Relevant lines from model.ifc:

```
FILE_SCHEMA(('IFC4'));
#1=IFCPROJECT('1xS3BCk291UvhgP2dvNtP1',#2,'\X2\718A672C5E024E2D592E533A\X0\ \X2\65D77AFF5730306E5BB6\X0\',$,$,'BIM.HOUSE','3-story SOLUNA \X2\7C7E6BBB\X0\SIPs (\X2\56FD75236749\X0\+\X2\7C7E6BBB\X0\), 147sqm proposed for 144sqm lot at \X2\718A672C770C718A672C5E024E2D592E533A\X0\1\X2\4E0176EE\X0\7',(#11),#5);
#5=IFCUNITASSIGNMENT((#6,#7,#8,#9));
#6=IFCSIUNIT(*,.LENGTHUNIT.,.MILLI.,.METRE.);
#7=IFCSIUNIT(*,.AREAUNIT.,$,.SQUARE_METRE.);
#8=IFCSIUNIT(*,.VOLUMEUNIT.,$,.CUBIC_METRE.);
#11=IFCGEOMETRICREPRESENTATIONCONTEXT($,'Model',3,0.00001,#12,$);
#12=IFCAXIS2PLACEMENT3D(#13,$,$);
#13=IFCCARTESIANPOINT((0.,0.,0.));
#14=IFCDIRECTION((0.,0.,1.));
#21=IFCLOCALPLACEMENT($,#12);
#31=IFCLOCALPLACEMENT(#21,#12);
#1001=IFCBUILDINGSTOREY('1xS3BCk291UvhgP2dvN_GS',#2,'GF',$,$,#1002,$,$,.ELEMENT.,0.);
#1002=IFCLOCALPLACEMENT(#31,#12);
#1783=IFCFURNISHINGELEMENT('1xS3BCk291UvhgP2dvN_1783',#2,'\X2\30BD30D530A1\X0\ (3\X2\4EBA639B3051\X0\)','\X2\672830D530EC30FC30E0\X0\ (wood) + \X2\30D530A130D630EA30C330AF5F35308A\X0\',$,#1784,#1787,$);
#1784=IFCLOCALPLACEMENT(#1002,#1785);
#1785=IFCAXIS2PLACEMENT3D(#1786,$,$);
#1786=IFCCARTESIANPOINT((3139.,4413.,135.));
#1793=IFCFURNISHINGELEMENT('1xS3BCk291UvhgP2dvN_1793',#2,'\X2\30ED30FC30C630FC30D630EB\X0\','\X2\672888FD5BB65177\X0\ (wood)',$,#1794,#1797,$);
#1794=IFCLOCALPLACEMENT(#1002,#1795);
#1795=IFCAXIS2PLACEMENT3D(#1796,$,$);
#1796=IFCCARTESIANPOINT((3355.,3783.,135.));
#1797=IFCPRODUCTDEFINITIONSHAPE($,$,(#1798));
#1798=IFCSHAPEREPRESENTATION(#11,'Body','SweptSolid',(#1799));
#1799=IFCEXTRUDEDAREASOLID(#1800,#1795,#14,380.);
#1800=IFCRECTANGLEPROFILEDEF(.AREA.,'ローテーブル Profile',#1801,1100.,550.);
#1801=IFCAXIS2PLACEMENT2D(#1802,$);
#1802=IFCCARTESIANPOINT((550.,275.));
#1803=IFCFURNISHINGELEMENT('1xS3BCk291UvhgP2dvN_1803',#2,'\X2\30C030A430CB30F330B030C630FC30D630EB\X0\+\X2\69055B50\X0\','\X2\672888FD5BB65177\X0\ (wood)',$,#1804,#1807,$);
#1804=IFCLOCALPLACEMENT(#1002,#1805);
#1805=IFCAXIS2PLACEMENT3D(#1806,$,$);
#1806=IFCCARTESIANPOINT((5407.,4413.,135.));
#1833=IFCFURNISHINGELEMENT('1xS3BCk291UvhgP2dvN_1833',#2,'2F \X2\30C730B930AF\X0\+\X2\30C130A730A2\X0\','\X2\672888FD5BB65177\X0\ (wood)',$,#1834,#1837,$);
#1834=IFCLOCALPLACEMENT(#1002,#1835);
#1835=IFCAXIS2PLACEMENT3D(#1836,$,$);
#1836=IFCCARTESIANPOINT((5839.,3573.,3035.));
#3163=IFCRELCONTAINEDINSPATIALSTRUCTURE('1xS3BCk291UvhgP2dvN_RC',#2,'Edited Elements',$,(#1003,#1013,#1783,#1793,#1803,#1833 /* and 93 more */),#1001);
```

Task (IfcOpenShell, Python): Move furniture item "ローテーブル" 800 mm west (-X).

```python
import ifcopenshell
import ifcopenshell.api.geometry
import ifcopenshell.util.placement
import ifcopenshell.util.unit

model = ifcopenshell.open("model.ifc")
unit_scale = ifcopenshell.util.unit.calculate_unit_scale(model)

item = model.by_guid("1xS3BCk291UvhgP2dvN_1793")
matrix = ifcopenshell.util.placement.get_local_placement(item.ObjectPlacement)
matrix[0, 3] -= 0.8 / unit_scale
ifcopenshell.api.geometry.edit_object_placement(model, product=item, matrix=matrix, is_si=False)

print(ifcopenshell.util.placement.get_local_placement(item.ObjectPlacement).round(3) + 0.0)

model.write("model_rev.ifc")
```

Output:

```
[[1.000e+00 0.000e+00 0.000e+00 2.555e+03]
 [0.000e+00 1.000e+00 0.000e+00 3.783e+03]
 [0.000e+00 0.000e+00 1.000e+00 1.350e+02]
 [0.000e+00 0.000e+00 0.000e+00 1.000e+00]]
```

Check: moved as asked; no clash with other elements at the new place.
